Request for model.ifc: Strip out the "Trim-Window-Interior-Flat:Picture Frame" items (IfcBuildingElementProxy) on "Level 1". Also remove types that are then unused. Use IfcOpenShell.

First a look at what the model holds.

```python
import ifcopenshell
import ifcopenshell.util.element

model = ifcopenshell.open("model.ifc")
print(model.schema)
storey = next(s for s in model.by_type("IfcBuildingStorey") if s.Name == "Level 1")
proxies = [e for e in ifcopenshell.util.element.get_decomposition(storey) if e.is_a("IfcBuildingElementProxy")]
seen = {}
for e in proxies:
    element_type = ifcopenshell.util.element.get_type(e)
    name = element_type.Name if element_type not in (None, e) else None
    seen[name] = seen.get(name, 0) + 1
for name, count in sorted(seen.items(), key=str):
    print(count, "x", name)
```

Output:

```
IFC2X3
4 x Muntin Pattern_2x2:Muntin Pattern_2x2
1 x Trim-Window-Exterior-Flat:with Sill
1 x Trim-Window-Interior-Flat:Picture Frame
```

```python
import ifcopenshell
import ifcopenshell.api.root
import ifcopenshell.util.element

model = ifcopenshell.open("model.ifc")

storey = next(s for s in model.by_type("IfcBuildingStorey") if s.Name == "Level 1")
proxies = [e for e in ifcopenshell.util.element.get_decomposition(storey) if e.is_a("IfcBuildingElementProxy")]
targets = [e for e in proxies if (t := ifcopenshell.util.element.get_type(e)) not in (None, e) and t.Name == "Trim-Window-Interior-Flat:Picture Frame"]
types = {ifcopenshell.util.element.get_type(e) for e in targets} - {None, *targets}

for e in targets:
    ifcopenshell.api.root.remove_product(model, product=e)
print(len(targets), "removed")

unused = [t for t in types if not ifcopenshell.util.element.get_types(t)]
for t in unused:
    ifcopenshell.api.root.remove_product(model, product=t)
print(len(unused), "unused types removed")

model.write("model_edited.ifc")
```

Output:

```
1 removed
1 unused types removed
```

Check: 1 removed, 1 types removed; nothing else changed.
